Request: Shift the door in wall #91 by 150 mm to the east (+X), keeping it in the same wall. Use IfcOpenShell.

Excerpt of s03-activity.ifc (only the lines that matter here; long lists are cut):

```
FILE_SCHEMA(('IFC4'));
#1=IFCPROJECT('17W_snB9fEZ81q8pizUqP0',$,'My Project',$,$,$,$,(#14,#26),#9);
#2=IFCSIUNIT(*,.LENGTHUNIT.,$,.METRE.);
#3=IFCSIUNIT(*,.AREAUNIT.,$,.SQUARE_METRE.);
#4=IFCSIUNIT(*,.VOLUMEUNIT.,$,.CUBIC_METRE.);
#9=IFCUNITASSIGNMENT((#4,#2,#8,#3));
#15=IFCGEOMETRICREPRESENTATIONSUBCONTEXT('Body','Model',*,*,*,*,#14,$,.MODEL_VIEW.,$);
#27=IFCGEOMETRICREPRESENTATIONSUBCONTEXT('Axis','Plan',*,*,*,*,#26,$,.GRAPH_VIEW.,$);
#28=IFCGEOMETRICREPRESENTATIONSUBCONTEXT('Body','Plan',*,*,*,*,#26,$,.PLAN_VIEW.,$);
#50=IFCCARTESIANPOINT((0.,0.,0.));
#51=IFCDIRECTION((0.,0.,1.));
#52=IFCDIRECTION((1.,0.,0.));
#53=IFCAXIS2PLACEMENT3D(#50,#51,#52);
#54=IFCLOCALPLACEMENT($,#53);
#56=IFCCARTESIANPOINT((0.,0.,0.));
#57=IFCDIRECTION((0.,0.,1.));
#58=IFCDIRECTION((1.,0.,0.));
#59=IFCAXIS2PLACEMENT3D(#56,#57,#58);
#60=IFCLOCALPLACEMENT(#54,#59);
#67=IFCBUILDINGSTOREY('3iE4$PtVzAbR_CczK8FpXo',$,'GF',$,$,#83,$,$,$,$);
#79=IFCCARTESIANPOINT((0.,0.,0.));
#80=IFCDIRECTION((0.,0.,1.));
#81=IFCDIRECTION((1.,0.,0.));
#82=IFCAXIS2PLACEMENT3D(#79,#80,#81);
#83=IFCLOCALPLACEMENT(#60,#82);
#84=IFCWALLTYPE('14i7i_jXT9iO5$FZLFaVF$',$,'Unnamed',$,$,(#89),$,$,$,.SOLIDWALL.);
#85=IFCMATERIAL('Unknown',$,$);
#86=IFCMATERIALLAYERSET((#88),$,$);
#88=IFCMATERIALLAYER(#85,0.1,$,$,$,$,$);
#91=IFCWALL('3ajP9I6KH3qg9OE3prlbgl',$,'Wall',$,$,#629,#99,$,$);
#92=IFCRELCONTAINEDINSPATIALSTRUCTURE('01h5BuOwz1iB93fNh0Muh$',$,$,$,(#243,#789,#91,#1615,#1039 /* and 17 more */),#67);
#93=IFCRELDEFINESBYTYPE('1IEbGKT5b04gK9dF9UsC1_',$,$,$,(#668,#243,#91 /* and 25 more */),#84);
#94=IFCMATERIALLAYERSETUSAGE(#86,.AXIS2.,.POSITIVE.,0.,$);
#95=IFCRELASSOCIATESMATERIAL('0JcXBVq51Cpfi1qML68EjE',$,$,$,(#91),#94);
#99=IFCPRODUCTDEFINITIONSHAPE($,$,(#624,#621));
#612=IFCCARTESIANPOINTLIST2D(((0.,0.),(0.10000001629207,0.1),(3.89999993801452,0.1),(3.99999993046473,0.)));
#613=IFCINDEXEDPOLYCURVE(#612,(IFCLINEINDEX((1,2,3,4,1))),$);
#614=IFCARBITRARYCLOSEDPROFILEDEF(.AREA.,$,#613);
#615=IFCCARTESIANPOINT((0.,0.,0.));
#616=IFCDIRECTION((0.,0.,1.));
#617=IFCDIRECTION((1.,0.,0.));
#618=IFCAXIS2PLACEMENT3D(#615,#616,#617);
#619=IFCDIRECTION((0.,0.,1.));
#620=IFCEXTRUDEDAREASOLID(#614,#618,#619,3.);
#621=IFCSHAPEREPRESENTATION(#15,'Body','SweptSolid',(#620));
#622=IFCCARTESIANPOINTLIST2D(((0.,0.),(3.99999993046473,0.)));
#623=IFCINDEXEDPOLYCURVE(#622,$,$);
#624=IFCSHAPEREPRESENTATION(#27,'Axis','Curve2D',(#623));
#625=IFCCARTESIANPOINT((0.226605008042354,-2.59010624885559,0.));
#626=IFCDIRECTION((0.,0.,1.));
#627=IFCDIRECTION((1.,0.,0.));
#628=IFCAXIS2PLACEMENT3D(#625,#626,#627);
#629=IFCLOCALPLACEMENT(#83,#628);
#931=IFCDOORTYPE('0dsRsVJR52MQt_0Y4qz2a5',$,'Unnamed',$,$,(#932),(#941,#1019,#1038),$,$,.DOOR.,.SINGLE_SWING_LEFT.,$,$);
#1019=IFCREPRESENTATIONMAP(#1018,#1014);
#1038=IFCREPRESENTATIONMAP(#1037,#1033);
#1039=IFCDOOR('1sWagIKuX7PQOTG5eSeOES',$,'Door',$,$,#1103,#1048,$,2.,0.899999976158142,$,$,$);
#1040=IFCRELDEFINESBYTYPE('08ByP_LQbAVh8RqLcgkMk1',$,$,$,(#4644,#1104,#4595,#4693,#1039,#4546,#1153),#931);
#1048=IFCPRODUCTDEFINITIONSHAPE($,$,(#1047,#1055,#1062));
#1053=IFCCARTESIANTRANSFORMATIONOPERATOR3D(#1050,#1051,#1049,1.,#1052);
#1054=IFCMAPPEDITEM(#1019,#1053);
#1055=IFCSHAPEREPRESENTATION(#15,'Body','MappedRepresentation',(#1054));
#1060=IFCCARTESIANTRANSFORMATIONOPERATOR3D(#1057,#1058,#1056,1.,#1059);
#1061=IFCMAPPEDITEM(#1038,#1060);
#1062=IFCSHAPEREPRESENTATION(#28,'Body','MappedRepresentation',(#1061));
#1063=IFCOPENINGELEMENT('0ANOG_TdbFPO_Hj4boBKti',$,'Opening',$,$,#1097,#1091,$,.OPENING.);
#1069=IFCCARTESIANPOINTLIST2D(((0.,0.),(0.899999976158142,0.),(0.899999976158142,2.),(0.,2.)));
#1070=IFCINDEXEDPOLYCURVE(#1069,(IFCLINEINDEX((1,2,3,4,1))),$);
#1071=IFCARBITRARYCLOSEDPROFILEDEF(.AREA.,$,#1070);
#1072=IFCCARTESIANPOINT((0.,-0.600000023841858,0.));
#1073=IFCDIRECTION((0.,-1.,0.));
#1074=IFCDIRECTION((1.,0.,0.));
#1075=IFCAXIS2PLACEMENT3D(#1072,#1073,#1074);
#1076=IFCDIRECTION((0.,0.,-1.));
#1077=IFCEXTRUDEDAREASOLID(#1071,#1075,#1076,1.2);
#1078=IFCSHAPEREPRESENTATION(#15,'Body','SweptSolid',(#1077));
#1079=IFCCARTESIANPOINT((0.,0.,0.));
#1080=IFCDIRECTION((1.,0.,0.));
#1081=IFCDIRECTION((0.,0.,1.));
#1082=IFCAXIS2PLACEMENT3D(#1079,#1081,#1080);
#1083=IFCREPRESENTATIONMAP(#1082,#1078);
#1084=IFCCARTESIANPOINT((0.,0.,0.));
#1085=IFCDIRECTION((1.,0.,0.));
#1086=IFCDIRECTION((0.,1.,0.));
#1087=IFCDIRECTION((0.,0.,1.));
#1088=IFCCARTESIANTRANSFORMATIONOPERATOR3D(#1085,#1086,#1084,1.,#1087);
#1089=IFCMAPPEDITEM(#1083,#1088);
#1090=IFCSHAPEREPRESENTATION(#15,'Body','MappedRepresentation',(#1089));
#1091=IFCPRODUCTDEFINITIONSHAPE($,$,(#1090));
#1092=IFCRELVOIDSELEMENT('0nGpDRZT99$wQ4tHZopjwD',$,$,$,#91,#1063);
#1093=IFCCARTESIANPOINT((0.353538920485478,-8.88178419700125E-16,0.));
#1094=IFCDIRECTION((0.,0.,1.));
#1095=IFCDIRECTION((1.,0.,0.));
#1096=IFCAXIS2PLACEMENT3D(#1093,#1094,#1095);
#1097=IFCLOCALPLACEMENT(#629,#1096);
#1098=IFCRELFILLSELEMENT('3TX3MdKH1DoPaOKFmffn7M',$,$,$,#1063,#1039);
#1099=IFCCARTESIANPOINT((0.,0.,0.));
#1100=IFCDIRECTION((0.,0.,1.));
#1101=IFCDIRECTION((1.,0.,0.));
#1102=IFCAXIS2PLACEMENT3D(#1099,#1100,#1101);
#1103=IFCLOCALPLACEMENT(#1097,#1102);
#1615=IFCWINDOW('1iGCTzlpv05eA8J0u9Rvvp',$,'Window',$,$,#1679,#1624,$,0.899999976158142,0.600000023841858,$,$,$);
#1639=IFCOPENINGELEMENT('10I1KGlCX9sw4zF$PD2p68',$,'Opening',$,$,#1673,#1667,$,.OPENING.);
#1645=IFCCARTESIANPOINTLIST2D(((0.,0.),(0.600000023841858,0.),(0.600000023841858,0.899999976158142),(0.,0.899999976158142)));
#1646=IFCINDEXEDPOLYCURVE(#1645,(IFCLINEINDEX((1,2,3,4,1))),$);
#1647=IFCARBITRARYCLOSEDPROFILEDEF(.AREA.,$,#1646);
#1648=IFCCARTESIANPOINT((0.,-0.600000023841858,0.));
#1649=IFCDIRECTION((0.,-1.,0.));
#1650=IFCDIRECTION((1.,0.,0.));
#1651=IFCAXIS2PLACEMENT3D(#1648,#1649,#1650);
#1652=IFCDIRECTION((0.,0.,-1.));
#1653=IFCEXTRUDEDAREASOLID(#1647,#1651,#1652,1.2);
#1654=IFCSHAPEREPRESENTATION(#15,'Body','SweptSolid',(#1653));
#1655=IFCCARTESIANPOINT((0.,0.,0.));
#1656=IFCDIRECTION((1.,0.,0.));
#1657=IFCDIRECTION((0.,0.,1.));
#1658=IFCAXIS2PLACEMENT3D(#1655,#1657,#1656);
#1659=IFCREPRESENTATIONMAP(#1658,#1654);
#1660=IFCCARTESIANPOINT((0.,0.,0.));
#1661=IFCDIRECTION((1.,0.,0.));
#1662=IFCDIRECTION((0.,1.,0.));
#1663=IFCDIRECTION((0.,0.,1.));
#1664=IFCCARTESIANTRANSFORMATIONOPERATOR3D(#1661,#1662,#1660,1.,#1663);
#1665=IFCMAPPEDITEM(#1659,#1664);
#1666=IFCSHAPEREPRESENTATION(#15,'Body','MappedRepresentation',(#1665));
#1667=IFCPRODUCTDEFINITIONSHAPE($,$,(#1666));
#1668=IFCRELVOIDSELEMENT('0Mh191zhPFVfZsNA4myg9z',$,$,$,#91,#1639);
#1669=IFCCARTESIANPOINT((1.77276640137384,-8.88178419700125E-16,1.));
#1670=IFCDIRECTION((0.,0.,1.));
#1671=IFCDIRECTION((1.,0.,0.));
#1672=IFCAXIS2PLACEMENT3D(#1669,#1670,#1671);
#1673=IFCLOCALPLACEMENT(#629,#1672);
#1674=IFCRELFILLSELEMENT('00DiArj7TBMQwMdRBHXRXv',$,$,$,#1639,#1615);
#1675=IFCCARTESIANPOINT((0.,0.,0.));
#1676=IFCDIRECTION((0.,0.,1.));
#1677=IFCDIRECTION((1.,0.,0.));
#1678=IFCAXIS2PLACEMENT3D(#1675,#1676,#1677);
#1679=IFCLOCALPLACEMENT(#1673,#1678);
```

```python
import ifcopenshell
import ifcopenshell.api.geometry
import ifcopenshell.util.placement
import ifcopenshell.util.unit

model = ifcopenshell.open("s03-activity.ifc")
unit_scale = ifcopenshell.util.unit.calculate_unit_scale(model)

door = model.by_id(1039)
opening = door.FillsVoids[0].RelatingOpeningElement
wall = opening.VoidsElements[0].RelatingBuildingElement

wall_matrix = ifcopenshell.util.placement.get_local_placement(wall.ObjectPlacement)
shift = wall_matrix[:3, 0] * 0.15 / unit_scale
before = ifcopenshell.util.placement.get_local_placement(door.ObjectPlacement)[:3, 3].copy()

# The door is placed relative to its opening, so it follows when the opening moves.
matrix = ifcopenshell.util.placement.get_local_placement(opening.ObjectPlacement)
matrix[:3, 3] += shift
ifcopenshell.api.geometry.edit_object_placement(
    model, product=opening, matrix=matrix, is_si=False, should_transform_children=True
)

after = ifcopenshell.util.placement.get_local_placement(door.ObjectPlacement)[:3, 3]
print("door moved by", (after - before).round(3) + 0.0)

model.write("s03-activity_edited.ifc")
```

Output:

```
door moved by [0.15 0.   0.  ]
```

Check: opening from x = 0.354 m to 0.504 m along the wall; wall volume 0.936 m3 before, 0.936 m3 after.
